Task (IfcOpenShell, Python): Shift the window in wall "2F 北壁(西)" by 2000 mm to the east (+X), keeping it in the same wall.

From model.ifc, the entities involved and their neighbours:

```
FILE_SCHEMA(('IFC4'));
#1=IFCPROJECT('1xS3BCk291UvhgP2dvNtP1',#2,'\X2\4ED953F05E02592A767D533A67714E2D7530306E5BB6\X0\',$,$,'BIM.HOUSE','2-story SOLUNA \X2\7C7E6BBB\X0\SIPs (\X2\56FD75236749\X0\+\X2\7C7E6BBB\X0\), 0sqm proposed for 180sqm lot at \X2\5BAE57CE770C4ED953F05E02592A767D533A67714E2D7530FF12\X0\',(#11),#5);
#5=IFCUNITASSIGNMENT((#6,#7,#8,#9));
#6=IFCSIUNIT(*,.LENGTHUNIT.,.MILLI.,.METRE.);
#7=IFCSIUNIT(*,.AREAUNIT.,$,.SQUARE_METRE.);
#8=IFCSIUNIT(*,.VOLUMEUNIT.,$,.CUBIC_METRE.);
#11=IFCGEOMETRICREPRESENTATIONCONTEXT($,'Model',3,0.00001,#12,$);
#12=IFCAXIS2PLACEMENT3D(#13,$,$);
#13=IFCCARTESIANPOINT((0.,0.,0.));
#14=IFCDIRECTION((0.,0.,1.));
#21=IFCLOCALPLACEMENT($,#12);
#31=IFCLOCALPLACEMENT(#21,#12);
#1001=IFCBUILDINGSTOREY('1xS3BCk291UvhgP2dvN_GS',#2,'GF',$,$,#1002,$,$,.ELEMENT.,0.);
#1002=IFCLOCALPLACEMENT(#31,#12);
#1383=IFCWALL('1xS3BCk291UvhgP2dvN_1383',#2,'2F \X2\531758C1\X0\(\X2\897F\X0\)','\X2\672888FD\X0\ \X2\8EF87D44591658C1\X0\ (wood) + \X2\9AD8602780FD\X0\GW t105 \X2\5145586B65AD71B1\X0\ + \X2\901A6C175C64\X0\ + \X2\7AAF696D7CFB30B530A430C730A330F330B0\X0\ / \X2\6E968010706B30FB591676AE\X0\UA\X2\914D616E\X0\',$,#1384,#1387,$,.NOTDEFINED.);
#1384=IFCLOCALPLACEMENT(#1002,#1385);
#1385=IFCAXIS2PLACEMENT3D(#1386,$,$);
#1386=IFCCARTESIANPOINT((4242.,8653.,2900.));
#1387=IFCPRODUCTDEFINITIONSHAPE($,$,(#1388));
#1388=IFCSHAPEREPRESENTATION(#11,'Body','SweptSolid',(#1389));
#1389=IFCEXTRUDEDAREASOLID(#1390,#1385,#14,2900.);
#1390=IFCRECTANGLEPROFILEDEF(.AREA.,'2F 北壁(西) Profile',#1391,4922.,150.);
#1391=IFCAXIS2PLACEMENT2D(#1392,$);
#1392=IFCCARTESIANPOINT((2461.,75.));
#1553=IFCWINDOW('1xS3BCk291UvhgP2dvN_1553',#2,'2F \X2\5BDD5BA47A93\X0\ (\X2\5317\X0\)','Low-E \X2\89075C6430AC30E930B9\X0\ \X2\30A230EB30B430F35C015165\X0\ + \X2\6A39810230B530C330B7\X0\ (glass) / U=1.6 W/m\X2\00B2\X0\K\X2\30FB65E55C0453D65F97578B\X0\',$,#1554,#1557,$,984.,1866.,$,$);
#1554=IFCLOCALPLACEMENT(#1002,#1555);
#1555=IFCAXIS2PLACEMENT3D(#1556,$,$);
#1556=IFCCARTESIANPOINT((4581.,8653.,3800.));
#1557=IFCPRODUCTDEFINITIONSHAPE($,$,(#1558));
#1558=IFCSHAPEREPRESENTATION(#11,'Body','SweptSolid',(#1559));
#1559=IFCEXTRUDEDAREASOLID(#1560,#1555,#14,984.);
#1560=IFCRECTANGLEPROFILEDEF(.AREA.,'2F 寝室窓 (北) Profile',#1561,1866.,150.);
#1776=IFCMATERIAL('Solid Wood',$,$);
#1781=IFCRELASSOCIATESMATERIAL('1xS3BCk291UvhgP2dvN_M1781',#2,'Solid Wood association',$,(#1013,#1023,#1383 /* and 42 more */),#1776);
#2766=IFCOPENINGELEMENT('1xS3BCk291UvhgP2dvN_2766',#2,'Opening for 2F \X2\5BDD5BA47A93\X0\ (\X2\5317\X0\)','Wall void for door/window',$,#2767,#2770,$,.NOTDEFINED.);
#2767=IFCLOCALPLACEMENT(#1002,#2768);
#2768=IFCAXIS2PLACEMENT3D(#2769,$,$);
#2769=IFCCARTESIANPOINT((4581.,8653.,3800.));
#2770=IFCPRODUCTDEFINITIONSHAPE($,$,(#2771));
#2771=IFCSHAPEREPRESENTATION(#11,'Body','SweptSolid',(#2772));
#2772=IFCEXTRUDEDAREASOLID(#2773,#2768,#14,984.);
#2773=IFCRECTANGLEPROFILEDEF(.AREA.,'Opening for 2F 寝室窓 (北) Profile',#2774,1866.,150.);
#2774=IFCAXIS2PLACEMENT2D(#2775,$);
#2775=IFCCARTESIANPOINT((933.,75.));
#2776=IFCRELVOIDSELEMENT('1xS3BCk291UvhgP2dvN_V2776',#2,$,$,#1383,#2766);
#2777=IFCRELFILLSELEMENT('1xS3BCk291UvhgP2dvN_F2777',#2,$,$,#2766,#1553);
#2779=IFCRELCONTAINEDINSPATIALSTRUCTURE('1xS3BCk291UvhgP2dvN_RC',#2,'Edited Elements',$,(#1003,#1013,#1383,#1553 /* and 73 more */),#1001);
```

```python
import ifcopenshell
import ifcopenshell.api.geometry
import ifcopenshell.util.placement
import ifcopenshell.util.unit

model = ifcopenshell.open("model.ifc")
unit_scale = ifcopenshell.util.unit.calculate_unit_scale(model)

window = model.by_id(1553)
opening = window.FillsVoids[0].RelatingOpeningElement
wall = opening.VoidsElements[0].RelatingBuildingElement

wall_matrix = ifcopenshell.util.placement.get_local_placement(wall.ObjectPlacement)
shift = wall_matrix[:3, 0] * 2 / unit_scale
before = ifcopenshell.util.placement.get_local_placement(window.ObjectPlacement)[:3, 3].copy()

# The window is not placed relative to its opening, so move both.
for product in (opening, window):
    matrix = ifcopenshell.util.placement.get_local_placement(product.ObjectPlacement)
    matrix[:3, 3] += shift
    ifcopenshell.api.geometry.edit_object_placement(model, product=product, matrix=matrix, is_si=False)

after = ifcopenshell.util.placement.get_local_placement(window.ObjectPlacement)[:3, 3]
print("window moved by", (after - before).round(3) + 0.0)

model.write("model_rev.ifc")
```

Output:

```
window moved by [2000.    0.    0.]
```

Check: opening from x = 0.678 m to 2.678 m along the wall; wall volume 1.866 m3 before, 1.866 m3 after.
